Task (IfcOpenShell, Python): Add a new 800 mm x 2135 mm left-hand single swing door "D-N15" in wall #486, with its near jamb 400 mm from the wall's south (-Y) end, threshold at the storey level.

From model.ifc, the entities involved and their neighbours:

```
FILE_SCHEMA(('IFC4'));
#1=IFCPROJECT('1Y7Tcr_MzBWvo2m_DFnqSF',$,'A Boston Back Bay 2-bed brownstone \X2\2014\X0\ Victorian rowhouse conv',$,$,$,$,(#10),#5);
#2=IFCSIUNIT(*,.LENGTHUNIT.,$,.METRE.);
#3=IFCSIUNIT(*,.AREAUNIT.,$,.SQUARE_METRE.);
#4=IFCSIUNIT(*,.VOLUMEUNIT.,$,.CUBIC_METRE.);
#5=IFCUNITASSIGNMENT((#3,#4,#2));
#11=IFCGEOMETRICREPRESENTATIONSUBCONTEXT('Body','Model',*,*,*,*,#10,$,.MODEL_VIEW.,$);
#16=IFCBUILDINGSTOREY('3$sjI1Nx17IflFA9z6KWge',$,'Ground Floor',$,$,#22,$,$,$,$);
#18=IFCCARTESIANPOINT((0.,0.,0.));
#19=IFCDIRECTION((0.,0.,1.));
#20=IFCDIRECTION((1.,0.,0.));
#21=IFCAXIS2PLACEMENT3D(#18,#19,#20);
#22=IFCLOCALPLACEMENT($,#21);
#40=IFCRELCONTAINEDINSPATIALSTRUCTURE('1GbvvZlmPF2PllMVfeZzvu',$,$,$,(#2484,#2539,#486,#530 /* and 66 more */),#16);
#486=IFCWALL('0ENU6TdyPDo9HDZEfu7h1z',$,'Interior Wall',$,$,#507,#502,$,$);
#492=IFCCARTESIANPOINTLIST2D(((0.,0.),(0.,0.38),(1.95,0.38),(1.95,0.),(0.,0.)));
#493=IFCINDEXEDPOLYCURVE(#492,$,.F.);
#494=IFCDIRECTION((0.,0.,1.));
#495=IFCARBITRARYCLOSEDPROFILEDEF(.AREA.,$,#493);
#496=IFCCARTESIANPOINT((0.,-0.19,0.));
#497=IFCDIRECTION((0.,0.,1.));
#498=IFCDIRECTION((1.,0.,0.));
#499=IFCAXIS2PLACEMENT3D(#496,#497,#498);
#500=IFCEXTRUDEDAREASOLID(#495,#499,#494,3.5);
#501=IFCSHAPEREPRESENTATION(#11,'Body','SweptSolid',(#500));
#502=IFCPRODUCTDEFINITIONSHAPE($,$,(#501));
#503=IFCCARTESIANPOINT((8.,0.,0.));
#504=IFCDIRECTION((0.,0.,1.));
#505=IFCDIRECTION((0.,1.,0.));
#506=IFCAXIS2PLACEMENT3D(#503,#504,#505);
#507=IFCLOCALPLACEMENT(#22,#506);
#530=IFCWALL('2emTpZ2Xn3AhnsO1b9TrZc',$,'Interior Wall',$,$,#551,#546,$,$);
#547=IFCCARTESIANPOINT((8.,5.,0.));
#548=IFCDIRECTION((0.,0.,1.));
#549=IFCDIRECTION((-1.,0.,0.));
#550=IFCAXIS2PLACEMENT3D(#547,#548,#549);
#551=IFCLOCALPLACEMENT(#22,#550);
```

```python
import numpy as np
import ifcopenshell
import ifcopenshell.api.feature
import ifcopenshell.api.geometry
import ifcopenshell.api.root
import ifcopenshell.api.spatial
import ifcopenshell.geom
import ifcopenshell.util.element
import ifcopenshell.util.placement
import ifcopenshell.util.representation
import ifcopenshell.util.shape
import ifcopenshell.util.unit

model = ifcopenshell.open("model.ifc")
unit_scale = ifcopenshell.util.unit.calculate_unit_scale(model)
settings = ifcopenshell.geom.settings()


def volume(element):
    """Net volume in cubic metres, openings subtracted."""
    shape = ifcopenshell.geom.create_shape(settings, element)
    return ifcopenshell.util.shape.get_volume(shape.geometry)


wall = model.by_id(486)
storey = ifcopenshell.util.element.get_container(wall, ifc_class="IfcBuildingStorey")
context = ifcopenshell.util.representation.get_context(model, "Model", "Body", "MODEL_VIEW")
before = volume(wall)

width, height, from_end, sill = 0.8, 2.135, 0.4, 0.0  # metres

# The wall runs along its own X axis, and the end named is its -X end.
wall_shape = ifcopenshell.geom.create_shape(settings, wall)
x, y, z = ifcopenshell.util.shape.get_vertices(wall_shape.geometry).T
start = x.min() + from_end
face, thickness = float(y.min()), float(y.max() - y.min())
wall_matrix = ifcopenshell.util.placement.get_local_placement(wall.ObjectPlacement)
level = ifcopenshell.util.placement.get_local_placement(storey.ObjectPlacement)[2, 3]


def in_wall(x, y):
    """Placement at x, y metres in the wall's axes, at sill height."""
    matrix = wall_matrix.copy()
    matrix[:, 3] = wall_matrix @ np.array([x / unit_scale, y / unit_scale, 0.0, 1.0])
    matrix[2, 3] = level + sill / unit_scale
    return matrix


# Opening: a box that overshoots both wall faces by 50 mm.
opening = ifcopenshell.api.root.create_entity(model, ifc_class="IfcOpeningElement", predefined_type="OPENING")
box = ifcopenshell.api.geometry.add_wall_representation(
    model, context=context, length=width, height=height, thickness=thickness + 0.1
)
ifcopenshell.api.geometry.assign_representation(model, product=opening, representation=box)
ifcopenshell.api.geometry.edit_object_placement(model, product=opening, matrix=in_wall(start, face - 0.05), is_si=False)
ifcopenshell.api.feature.add_feature(model, feature=opening, element=wall)

door = ifcopenshell.api.root.create_entity(model, ifc_class="IfcDoor", name="D-N15", predefined_type="DOOR")
door.OverallWidth, door.OverallHeight = width / unit_scale, height / unit_scale
door.OperationType = "SINGLE_SWING_LEFT"
body = ifcopenshell.api.geometry.add_door_representation(
    model,
    context=context,
    overall_width=door.OverallWidth,
    overall_height=door.OverallHeight,
    operation_type="SINGLE_SWING_LEFT",
    lining_properties={"LiningDepth": thickness / unit_scale, "ThresholdDepth": thickness / unit_scale},
)
ifcopenshell.api.geometry.assign_representation(model, product=door, representation=body)
ifcopenshell.api.spatial.assign_container(model, products=[door], relating_structure=storey)
ifcopenshell.api.feature.add_filling(model, opening=opening, element=door)

# The lining spans the wall, so the door starts at the wall face.
ifcopenshell.api.geometry.edit_object_placement(model, product=door, matrix=in_wall(start, face), is_si=False)

after = volume(wall)

print(f"wall volume {before:.3f} -> {after:.3f} m3")

model.write("model_rev.ifc")
```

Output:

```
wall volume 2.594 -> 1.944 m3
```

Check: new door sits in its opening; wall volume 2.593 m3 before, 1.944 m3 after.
